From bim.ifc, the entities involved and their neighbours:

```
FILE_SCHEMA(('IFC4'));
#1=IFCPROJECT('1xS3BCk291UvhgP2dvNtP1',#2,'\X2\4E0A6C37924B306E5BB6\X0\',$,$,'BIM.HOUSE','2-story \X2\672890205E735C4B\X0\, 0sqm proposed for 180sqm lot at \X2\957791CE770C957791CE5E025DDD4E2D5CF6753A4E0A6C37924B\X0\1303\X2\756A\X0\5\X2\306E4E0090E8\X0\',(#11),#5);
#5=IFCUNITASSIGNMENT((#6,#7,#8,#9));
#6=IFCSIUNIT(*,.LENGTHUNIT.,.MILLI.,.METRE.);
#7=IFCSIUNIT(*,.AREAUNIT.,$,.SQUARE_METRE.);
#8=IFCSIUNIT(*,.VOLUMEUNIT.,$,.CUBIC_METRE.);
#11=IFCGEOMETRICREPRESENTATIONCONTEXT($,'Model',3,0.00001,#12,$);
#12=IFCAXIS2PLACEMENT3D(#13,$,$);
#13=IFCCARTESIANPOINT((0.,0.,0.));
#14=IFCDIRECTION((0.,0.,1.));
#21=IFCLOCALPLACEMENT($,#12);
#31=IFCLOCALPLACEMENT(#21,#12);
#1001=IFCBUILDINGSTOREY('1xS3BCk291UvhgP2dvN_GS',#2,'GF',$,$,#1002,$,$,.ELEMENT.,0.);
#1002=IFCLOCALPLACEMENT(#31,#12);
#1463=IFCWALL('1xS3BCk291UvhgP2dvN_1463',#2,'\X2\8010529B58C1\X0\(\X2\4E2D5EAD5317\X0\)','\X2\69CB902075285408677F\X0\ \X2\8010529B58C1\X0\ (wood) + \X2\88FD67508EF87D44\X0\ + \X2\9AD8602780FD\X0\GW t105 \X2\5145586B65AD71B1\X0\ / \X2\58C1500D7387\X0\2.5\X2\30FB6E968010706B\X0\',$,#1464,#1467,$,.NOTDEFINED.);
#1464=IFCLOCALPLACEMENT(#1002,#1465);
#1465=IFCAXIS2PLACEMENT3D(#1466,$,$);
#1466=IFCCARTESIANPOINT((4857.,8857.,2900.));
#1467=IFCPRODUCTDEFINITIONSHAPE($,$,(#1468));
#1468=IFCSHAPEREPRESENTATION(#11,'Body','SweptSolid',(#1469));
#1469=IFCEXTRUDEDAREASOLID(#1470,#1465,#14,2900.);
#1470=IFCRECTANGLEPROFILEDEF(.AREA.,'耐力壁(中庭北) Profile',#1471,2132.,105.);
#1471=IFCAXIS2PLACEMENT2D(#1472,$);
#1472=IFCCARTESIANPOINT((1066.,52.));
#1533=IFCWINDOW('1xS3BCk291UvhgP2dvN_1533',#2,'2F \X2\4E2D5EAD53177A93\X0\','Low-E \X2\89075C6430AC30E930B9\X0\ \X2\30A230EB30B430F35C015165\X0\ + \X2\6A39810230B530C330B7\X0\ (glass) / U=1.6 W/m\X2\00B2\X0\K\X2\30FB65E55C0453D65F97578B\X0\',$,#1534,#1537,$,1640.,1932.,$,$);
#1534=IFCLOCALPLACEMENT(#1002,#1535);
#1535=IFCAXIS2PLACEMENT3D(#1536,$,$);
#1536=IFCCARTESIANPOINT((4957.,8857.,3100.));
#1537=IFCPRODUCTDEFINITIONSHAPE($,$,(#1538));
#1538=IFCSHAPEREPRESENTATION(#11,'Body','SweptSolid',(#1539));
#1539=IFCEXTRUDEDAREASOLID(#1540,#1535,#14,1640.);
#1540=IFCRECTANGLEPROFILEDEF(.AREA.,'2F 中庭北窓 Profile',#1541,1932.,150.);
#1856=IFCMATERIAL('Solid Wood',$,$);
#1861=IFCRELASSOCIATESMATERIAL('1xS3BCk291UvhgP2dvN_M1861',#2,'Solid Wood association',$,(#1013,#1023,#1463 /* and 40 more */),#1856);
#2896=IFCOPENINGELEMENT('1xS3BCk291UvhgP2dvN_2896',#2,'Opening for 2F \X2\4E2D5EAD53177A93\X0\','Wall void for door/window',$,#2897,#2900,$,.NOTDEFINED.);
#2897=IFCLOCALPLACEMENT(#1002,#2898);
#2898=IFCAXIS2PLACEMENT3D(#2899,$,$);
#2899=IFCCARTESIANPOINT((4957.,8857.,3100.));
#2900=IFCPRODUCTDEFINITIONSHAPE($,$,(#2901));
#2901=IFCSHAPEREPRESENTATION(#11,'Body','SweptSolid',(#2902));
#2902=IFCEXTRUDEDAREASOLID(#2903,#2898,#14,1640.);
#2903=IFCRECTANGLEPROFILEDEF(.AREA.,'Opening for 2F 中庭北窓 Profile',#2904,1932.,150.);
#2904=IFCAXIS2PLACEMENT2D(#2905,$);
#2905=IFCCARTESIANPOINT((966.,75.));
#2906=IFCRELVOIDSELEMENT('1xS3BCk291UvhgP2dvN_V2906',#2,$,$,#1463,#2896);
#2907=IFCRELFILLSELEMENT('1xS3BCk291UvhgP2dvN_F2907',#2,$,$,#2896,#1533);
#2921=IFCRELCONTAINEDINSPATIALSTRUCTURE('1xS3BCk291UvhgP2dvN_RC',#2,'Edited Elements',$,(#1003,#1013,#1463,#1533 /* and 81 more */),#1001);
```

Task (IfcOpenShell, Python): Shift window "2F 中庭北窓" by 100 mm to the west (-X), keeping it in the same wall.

```python
import ifcopenshell
import ifcopenshell.api.geometry
import ifcopenshell.util.placement

model = ifcopenshell.open("bim.ifc")

window = model.by_guid("1xS3BCk291UvhgP2dvN_1533")
opening = window.FillsVoids[0].RelatingOpeningElement
wall = opening.VoidsElements[0].RelatingBuildingElement

wall_matrix = ifcopenshell.util.placement.get_local_placement(wall.ObjectPlacement)
shift = wall_matrix[:3, 0] * -100.0
before = ifcopenshell.util.placement.get_local_placement(window.ObjectPlacement)[:3, 3].copy()

# The window is not placed relative to its opening, so move both.
for product in (opening, window):
    matrix = ifcopenshell.util.placement.get_local_placement(product.ObjectPlacement)
    matrix[:3, 3] += shift
    ifcopenshell.api.geometry.edit_object_placement(model, product=product, matrix=matrix, is_si=False)

after = ifcopenshell.util.placement.get_local_placement(window.ObjectPlacement)[:3, 3]
print("window moved by", (after - before).round(3) + 0.0)

model.write("bim_edited.ifc")
```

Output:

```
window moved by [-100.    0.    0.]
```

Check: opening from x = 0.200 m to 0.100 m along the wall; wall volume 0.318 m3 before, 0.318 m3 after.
